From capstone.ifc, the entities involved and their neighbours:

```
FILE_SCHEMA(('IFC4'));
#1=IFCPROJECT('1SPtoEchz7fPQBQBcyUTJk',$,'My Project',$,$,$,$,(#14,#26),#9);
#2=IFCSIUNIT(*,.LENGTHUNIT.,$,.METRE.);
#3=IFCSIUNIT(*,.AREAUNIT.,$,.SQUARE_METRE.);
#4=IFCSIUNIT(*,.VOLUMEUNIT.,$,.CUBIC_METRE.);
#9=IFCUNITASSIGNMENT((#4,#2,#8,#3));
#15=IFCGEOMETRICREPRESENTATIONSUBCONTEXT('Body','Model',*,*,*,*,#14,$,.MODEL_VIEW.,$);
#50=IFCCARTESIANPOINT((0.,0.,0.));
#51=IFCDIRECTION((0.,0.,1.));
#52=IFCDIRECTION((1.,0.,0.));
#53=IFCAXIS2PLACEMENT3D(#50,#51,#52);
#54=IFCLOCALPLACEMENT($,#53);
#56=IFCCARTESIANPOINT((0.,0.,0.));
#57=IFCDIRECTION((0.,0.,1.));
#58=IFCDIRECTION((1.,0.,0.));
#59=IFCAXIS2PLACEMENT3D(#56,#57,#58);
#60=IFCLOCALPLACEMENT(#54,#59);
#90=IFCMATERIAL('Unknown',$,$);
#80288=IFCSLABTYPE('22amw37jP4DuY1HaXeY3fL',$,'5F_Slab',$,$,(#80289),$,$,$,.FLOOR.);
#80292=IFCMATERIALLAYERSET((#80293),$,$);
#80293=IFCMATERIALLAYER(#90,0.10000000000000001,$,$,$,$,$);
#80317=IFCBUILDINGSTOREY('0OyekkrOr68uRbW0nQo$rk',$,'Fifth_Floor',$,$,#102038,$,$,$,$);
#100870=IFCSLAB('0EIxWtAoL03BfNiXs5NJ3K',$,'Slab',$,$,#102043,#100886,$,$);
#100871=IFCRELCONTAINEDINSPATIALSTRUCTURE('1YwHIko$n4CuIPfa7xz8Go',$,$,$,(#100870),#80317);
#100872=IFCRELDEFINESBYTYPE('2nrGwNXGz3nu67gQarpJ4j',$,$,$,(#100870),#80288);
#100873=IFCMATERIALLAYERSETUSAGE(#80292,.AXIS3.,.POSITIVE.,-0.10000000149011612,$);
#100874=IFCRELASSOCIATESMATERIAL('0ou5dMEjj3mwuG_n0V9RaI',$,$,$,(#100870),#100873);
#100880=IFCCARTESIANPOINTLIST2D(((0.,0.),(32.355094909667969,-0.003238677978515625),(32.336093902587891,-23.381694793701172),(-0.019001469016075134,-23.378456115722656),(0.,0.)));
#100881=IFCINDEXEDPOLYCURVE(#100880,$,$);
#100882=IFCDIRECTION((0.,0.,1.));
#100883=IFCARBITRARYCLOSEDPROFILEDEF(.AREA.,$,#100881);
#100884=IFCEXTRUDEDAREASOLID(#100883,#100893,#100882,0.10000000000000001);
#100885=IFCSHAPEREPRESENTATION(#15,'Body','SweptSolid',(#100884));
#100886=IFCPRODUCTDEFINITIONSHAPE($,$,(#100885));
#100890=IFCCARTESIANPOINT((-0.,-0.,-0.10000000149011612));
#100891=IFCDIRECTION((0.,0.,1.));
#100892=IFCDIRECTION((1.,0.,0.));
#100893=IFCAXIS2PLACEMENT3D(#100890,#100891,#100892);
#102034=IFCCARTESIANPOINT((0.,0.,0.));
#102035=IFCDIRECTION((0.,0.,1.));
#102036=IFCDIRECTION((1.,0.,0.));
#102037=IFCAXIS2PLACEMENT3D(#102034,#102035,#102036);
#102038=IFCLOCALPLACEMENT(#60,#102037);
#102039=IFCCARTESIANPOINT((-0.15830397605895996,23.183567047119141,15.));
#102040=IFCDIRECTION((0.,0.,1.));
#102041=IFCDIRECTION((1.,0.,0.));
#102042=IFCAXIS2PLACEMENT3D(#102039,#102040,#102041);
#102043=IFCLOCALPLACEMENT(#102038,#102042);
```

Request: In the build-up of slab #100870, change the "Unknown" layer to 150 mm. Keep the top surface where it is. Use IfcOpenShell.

```python
import ifcopenshell
import ifcopenshell.util.element
import ifcopenshell.util.representation

model = ifcopenshell.open("capstone.ifc")

layer_set = model.by_id(80292)
layer = next(l for l in layer_set.MaterialLayers if l.Material and l.Material.Name == "Unknown")
change = 0.15 - layer.LayerThickness
layer.LayerThickness += change

# Geometry does not follow the layer set by itself.
slabs = [e for e in ifcopenshell.util.element.get_elements_by_material(model, layer_set) if e.is_a("IfcSlab")]
for slab in sorted(slabs, key=lambda e: e.id()):
    body = ifcopenshell.util.representation.get_representation(slab, "Model", "Body")
    solid = body.Items[0]
    old_depth = solid.Depth
    solid.Depth += change
    # Extruded upwards: lower the start of the extrusion so the top stays.
    x, y, z = solid.Position.Location.Coordinates
    solid.Position.Location = model.createIfcCartesianPoint((x, y, z - change))
    print(slab.id(), f"{old_depth:g} -> {solid.Depth:g}")

# The layers are counted up from the underside, which has moved.
for usage in {ifcopenshell.util.element.get_material(slab) for slab in slabs}:
    usage.OffsetFromReferenceLine -= change

model.write("capstone_updated.ifc")
```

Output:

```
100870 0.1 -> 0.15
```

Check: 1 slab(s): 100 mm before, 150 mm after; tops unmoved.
